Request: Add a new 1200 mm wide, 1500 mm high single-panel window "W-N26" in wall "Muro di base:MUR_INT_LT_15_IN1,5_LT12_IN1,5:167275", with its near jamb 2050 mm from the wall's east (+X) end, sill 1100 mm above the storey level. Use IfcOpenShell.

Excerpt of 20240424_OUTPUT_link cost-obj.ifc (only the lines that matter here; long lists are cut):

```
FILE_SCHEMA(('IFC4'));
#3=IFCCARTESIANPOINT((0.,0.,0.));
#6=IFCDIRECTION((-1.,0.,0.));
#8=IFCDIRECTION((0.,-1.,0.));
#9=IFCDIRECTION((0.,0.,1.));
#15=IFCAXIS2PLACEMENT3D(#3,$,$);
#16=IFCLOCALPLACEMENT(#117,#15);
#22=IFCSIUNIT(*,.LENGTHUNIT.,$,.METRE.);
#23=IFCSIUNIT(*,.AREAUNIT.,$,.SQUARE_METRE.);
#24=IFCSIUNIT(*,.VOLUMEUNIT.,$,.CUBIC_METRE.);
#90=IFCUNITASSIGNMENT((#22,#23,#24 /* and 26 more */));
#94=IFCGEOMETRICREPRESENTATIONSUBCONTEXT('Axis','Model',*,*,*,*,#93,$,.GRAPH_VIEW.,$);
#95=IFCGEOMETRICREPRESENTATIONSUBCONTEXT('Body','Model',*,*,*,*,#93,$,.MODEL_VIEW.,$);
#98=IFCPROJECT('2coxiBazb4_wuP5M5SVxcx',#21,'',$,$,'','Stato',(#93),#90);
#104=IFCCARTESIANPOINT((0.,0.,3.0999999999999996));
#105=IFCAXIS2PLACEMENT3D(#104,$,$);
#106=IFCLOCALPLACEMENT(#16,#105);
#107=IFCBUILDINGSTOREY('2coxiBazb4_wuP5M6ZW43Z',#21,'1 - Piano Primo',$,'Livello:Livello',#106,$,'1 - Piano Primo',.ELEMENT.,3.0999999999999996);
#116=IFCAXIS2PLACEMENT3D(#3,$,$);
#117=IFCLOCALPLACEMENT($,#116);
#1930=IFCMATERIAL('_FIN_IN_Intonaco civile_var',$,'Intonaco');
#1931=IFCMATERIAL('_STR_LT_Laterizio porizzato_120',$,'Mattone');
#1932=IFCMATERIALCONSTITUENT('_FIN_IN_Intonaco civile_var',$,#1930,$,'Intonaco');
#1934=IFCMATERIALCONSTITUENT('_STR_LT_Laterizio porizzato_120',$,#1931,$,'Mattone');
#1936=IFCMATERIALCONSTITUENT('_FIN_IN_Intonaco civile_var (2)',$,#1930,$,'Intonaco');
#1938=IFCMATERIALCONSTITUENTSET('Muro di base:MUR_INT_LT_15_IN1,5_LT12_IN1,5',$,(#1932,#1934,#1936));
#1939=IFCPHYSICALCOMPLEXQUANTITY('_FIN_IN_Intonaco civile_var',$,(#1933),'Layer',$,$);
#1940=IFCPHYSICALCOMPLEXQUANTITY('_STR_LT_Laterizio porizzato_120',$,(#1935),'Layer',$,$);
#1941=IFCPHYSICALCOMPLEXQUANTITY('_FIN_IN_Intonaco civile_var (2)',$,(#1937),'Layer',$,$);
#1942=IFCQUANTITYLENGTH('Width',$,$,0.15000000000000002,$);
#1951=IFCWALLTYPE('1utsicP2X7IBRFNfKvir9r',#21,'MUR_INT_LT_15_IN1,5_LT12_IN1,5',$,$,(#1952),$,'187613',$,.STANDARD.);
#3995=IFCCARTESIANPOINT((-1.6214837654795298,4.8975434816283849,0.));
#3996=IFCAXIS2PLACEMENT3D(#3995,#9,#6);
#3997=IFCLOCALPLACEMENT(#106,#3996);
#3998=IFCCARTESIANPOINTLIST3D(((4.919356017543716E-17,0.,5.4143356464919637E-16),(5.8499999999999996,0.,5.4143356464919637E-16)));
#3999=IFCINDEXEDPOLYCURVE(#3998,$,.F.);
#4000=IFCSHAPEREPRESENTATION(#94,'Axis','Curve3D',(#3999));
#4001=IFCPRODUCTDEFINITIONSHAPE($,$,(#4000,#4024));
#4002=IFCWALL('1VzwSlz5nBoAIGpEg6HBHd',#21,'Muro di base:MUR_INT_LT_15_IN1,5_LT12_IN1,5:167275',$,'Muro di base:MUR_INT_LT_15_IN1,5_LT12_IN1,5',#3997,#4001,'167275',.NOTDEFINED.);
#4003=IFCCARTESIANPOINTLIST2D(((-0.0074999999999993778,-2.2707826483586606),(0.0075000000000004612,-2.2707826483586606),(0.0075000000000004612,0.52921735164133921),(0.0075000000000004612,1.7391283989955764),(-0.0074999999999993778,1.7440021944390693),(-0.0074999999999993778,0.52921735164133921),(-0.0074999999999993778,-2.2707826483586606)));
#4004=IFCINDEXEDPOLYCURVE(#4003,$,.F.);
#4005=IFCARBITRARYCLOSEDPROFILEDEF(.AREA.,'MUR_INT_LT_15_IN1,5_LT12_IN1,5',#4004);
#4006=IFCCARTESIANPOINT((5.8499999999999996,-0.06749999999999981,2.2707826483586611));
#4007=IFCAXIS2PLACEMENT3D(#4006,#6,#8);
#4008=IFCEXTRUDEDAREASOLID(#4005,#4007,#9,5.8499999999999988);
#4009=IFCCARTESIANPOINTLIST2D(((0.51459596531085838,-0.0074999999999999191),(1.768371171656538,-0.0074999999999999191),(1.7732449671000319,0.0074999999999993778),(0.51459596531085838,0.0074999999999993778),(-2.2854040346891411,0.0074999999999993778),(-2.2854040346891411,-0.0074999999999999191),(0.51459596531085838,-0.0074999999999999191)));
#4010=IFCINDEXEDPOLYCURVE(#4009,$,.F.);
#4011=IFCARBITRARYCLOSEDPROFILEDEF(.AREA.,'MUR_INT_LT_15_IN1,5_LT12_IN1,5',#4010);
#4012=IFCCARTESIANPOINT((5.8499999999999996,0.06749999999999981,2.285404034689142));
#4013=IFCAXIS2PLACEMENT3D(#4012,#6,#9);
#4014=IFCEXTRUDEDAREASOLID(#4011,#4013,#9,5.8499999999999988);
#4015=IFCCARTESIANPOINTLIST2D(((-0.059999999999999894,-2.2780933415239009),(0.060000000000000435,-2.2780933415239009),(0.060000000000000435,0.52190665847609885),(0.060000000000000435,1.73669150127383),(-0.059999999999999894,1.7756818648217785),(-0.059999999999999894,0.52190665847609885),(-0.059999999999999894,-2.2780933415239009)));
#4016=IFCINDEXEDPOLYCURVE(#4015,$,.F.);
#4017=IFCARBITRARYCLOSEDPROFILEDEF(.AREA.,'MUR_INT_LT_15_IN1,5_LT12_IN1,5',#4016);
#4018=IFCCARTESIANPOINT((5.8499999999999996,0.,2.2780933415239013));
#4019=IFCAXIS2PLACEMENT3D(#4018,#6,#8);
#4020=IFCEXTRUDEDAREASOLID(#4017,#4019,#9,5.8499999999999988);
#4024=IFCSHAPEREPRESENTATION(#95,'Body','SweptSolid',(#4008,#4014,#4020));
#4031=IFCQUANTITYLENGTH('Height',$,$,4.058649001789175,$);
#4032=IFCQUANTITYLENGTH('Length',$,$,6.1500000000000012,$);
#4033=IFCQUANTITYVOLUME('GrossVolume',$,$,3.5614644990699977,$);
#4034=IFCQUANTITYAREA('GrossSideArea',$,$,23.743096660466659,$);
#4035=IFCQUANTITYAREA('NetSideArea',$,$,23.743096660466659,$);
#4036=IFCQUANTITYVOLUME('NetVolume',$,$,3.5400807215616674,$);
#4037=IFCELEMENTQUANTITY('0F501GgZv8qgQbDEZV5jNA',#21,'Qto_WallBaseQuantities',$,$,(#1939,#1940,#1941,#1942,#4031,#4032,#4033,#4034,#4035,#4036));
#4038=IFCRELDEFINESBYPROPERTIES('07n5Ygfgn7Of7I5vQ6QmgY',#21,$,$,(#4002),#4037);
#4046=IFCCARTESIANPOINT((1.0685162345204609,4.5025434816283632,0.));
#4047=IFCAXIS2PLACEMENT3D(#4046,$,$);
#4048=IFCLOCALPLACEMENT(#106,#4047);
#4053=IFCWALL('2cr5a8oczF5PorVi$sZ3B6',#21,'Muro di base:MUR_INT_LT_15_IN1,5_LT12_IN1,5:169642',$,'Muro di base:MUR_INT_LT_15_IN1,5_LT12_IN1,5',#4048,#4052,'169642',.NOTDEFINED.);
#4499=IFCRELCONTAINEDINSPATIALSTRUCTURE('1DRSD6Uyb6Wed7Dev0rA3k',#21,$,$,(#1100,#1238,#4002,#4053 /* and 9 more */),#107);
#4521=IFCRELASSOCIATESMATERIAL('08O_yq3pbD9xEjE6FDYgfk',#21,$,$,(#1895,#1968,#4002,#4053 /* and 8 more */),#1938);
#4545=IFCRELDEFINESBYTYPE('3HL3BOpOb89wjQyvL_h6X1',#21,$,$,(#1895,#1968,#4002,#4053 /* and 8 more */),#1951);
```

```python
import numpy as np
import ifcopenshell
import ifcopenshell.api.feature
import ifcopenshell.api.geometry
import ifcopenshell.api.pset
import ifcopenshell.api.root
import ifcopenshell.api.spatial
import ifcopenshell.geom
import ifcopenshell.util.element
import ifcopenshell.util.placement
import ifcopenshell.util.representation
import ifcopenshell.util.shape
import ifcopenshell.util.unit

model = ifcopenshell.open("20240424_OUTPUT_link cost-obj.ifc")
unit_scale = ifcopenshell.util.unit.calculate_unit_scale(model)
area_scale = ifcopenshell.util.unit.calculate_unit_scale(model, "AREAUNIT")
volume_scale = ifcopenshell.util.unit.calculate_unit_scale(model, "VOLUMEUNIT")
settings = ifcopenshell.geom.settings()


def volume(element):
    """Net volume in cubic metres, openings subtracted."""
    shape = ifcopenshell.geom.create_shape(settings, element)
    return ifcopenshell.util.shape.get_volume(shape.geometry)


wall = model.by_guid("1VzwSlz5nBoAIGpEg6HBHd")
storey = ifcopenshell.util.element.get_container(wall, ifc_class="IfcBuildingStorey")
context = ifcopenshell.util.representation.get_context(model, "Model", "Body", "MODEL_VIEW")
before = volume(wall)

width, height, from_end, sill = 1.2, 1.5, 2.05, 1.1  # metres

# The wall runs along its own X axis, and the end named is its -X end.
wall_shape = ifcopenshell.geom.create_shape(settings, wall)
x, y, z = ifcopenshell.util.shape.get_vertices(wall_shape.geometry).T
start = x.min() + from_end
face, thickness = float(y.min()), float(y.max() - y.min())
wall_matrix = ifcopenshell.util.placement.get_local_placement(wall.ObjectPlacement)
level = ifcopenshell.util.placement.get_local_placement(storey.ObjectPlacement)[2, 3]


def in_wall(x, y):
    """Placement at x, y metres in the wall's axes, at sill height."""
    matrix = wall_matrix.copy()
    matrix[:, 3] = wall_matrix @ np.array([x / unit_scale, y / unit_scale, 0.0, 1.0])
    matrix[2, 3] = level + sill / unit_scale
    return matrix


# Opening: a box that overshoots both wall faces by 50 mm.
opening = ifcopenshell.api.root.create_entity(model, ifc_class="IfcOpeningElement", predefined_type="OPENING")
box = ifcopenshell.api.geometry.add_wall_representation(
    model, context=context, length=width, height=height, thickness=thickness + 0.1
)
ifcopenshell.api.geometry.assign_representation(model, product=opening, representation=box)
ifcopenshell.api.geometry.edit_object_placement(model, product=opening, matrix=in_wall(start, face - 0.05), is_si=False)
ifcopenshell.api.feature.add_feature(model, feature=opening, element=wall)

window = ifcopenshell.api.root.create_entity(model, ifc_class="IfcWindow", name="W-N26", predefined_type="WINDOW")
window.OverallWidth, window.OverallHeight = width / unit_scale, height / unit_scale
window.PartitioningType = "SINGLE_PANEL"
body = ifcopenshell.api.geometry.add_window_representation(
    model,
    context=context,
    overall_width=window.OverallWidth,
    overall_height=window.OverallHeight,
    partition_type="SINGLE_PANEL",
)
ifcopenshell.api.geometry.assign_representation(model, product=window, representation=body)
ifcopenshell.api.spatial.assign_container(model, products=[window], relating_structure=storey)
ifcopenshell.api.feature.add_filling(model, opening=opening, element=window)

# Centre the window in the wall's thickness.
ifcopenshell.api.geometry.edit_object_placement(model, product=window, matrix=in_wall(start, face), is_si=False)
window_shape = ifcopenshell.geom.create_shape(settings, window)
depth = ifcopenshell.util.shape.get_vertices(window_shape.geometry)[:, 1]
offset = face + thickness / 2 - (depth.min() + depth.max()) / 2
ifcopenshell.api.geometry.edit_object_placement(model, product=window, matrix=in_wall(start, offset), is_si=False)

after = volume(wall)

# Update the wall's stored quantities.
qto = model.by_id(ifcopenshell.util.element.get_pset(wall, "Qto_WallBaseQuantities", should_inherit=False)["id"])
ifcopenshell.api.pset.edit_qto(model, qto=qto, properties={
    "NetSideArea": after / thickness / area_scale,
    "NetVolume": after / volume_scale,
})

print(f"wall volume {before:.3f} -> {after:.3f} m3")

model.write("20240424_OUTPUT_link cost-obj_v2.ifc")
```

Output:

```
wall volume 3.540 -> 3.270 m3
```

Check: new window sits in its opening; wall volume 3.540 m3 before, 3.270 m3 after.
